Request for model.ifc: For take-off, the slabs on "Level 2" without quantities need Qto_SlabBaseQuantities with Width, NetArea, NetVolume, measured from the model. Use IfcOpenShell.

First a look at what the model holds.

```python
import ifcopenshell
import ifcopenshell.util.element
import ifcopenshell.util.unit

model = ifcopenshell.open("model.ifc")
print(model.schema)
for unit_type in ("LENGTHUNIT", "AREAUNIT", "VOLUMEUNIT"):
    print(unit_type, ifcopenshell.util.unit.calculate_unit_scale(model, unit_type))
storey = next(s for s in model.by_type("IfcBuildingStorey") if s.Name == "Level 2")
slabs = [e for e in ifcopenshell.util.element.get_decomposition(storey) if e.is_a("IfcSlab")]
for e in sorted(slabs, key=lambda e: e.id()):
    print(e.id(), e.is_a(), e.Name, list(ifcopenshell.util.element.get_psets(e, qtos_only=True)), sep=" | ")
```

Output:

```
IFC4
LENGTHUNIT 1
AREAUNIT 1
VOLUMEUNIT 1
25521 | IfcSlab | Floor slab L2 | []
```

```python
import ifcopenshell
import ifcopenshell.api.pset
import ifcopenshell.geom
import ifcopenshell.util.element
import ifcopenshell.util.shape
import ifcopenshell.util.unit

model = ifcopenshell.open("model.ifc")
unit_scale = ifcopenshell.util.unit.calculate_unit_scale(model)
area_scale = ifcopenshell.util.unit.calculate_unit_scale(model, "AREAUNIT")
volume_scale = ifcopenshell.util.unit.calculate_unit_scale(model, "VOLUMEUNIT")
settings = ifcopenshell.geom.settings()

storey = next(s for s in model.by_type("IfcBuildingStorey") if s.Name == "Level 2")
slabs = [e for e in ifcopenshell.util.element.get_decomposition(storey) if e.is_a("IfcSlab")]

for e in sorted(slabs, key=lambda e: e.id()):
    if ifcopenshell.util.element.get_psets(e, qtos_only=True, should_inherit=False):
        continue
    # Geometry comes back in metres, in the element's own axes.
    shape = ifcopenshell.geom.create_shape(settings, e)
    values = {
        "Width": ifcopenshell.util.shape.get_z(shape.geometry) / unit_scale,
        "NetArea": ifcopenshell.util.shape.get_footprint_area(shape.geometry) / area_scale,
        "NetVolume": ifcopenshell.util.shape.get_volume(shape.geometry) / volume_scale,
    }
    qto = ifcopenshell.api.pset.add_qto(model, product=e, name="Qto_SlabBaseQuantities")
    ifcopenshell.api.pset.edit_qto(model, qto=qto, properties=values)
    print(e.id(), {k: round(v, 3) for k, v in values.items()})

model.write("model_updated.ifc")
```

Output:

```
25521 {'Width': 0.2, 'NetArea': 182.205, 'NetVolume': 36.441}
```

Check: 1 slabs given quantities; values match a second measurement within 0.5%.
